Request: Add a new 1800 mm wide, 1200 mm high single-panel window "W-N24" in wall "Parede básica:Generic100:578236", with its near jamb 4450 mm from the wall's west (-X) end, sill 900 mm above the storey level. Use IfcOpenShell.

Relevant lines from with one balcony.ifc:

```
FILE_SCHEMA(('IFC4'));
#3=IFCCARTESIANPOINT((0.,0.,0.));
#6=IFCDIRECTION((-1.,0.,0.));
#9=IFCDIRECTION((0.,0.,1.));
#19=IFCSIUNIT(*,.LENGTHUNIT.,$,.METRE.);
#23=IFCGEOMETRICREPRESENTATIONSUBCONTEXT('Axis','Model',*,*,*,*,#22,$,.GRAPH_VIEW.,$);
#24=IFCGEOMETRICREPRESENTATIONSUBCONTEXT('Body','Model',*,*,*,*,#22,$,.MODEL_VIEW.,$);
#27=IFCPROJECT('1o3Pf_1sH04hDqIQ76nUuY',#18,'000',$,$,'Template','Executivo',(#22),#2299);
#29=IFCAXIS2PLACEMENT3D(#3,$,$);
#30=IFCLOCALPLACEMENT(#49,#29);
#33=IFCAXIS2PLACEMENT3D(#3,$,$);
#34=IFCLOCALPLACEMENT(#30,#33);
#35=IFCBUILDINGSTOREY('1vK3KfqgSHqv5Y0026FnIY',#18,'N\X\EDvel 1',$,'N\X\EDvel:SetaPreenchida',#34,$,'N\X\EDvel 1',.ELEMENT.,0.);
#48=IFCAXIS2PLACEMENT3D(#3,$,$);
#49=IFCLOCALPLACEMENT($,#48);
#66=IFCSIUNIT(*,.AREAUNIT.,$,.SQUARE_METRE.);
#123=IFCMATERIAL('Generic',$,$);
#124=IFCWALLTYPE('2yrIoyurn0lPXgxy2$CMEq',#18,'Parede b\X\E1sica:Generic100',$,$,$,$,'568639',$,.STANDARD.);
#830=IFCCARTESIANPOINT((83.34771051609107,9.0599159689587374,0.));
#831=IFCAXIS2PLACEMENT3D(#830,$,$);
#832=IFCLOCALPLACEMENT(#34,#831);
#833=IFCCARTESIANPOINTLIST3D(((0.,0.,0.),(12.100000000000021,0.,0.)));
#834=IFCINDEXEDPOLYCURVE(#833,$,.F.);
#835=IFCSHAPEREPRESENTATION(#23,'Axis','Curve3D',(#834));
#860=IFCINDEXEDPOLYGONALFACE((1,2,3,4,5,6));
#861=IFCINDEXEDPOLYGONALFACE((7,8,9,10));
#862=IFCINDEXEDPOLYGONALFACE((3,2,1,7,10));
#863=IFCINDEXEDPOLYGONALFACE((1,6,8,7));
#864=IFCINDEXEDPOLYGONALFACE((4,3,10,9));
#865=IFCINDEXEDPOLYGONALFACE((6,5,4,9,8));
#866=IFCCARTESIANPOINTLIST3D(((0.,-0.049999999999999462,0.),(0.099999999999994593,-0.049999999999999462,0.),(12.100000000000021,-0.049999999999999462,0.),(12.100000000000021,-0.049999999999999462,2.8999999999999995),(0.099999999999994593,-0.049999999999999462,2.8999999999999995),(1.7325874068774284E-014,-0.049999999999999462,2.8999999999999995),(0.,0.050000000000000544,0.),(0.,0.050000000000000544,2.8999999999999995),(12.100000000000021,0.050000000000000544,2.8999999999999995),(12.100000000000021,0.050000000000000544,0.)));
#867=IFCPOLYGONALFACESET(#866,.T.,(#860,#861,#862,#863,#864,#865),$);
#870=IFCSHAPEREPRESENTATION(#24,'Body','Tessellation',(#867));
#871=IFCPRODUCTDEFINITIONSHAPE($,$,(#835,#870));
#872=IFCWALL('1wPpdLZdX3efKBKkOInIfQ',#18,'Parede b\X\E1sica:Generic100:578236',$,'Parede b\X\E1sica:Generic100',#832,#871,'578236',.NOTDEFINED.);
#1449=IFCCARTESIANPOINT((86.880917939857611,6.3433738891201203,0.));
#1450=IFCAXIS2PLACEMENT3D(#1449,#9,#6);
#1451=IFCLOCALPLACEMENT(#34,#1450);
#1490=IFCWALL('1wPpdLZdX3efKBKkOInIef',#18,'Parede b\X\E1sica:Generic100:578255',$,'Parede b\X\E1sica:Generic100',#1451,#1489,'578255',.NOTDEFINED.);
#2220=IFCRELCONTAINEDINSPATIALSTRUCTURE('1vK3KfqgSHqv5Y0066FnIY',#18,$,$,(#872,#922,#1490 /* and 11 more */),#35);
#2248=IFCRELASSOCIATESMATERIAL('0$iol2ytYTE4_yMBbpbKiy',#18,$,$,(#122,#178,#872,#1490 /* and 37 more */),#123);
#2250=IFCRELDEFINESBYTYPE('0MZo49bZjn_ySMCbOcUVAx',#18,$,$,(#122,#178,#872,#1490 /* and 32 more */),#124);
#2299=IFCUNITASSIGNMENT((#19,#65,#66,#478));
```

```python
import numpy as np
import ifcopenshell
import ifcopenshell.api.feature
import ifcopenshell.api.geometry
import ifcopenshell.api.root
import ifcopenshell.api.spatial
import ifcopenshell.geom
import ifcopenshell.util.element
import ifcopenshell.util.placement
import ifcopenshell.util.representation
import ifcopenshell.util.shape
import ifcopenshell.util.unit

model = ifcopenshell.open("with one balcony.ifc")
unit_scale = ifcopenshell.util.unit.calculate_unit_scale(model)
settings = ifcopenshell.geom.settings()


def volume(element):
    """Net volume in cubic metres, openings subtracted."""
    shape = ifcopenshell.geom.create_shape(settings, element)
    return ifcopenshell.util.shape.get_volume(shape.geometry)


wall = model.by_guid("1wPpdLZdX3efKBKkOInIfQ")
storey = ifcopenshell.util.element.get_container(wall, ifc_class="IfcBuildingStorey")
context = ifcopenshell.util.representation.get_context(model, "Model", "Body", "MODEL_VIEW")
before = volume(wall)

width, height, from_end, sill = 1.8, 1.2, 4.45, 0.9  # metres

# The wall runs along its own X axis, and the end named is its -X end.
wall_shape = ifcopenshell.geom.create_shape(settings, wall)
x, y, z = ifcopenshell.util.shape.get_vertices(wall_shape.geometry).T
start = x.min() + from_end
face, thickness = float(y.min()), float(y.max() - y.min())
wall_matrix = ifcopenshell.util.placement.get_local_placement(wall.ObjectPlacement)
level = ifcopenshell.util.placement.get_local_placement(storey.ObjectPlacement)[2, 3]


def in_wall(x, y):
    """Placement at x, y metres in the wall's axes, at sill height."""
    matrix = wall_matrix.copy()
    matrix[:, 3] = wall_matrix @ np.array([x / unit_scale, y / unit_scale, 0.0, 1.0])
    matrix[2, 3] = level + sill / unit_scale
    return matrix


# Opening: a box that overshoots both wall faces by 50 mm.
opening = ifcopenshell.api.root.create_entity(model, ifc_class="IfcOpeningElement", predefined_type="OPENING")
box = ifcopenshell.api.geometry.add_wall_representation(
    model, context=context, length=width, height=height, thickness=thickness + 0.1
)
ifcopenshell.api.geometry.assign_representation(model, product=opening, representation=box)
ifcopenshell.api.geometry.edit_object_placement(model, product=opening, matrix=in_wall(start, face - 0.05), is_si=False)
ifcopenshell.api.feature.add_feature(model, feature=opening, element=wall)

window = ifcopenshell.api.root.create_entity(model, ifc_class="IfcWindow", name="W-N24", predefined_type="WINDOW")
window.OverallWidth, window.OverallHeight = width / unit_scale, height / unit_scale
window.PartitioningType = "SINGLE_PANEL"
body = ifcopenshell.api.geometry.add_window_representation(
    model,
    context=context,
    overall_width=window.OverallWidth,
    overall_height=window.OverallHeight,
    partition_type="SINGLE_PANEL",
)
ifcopenshell.api.geometry.assign_representation(model, product=window, representation=body)
ifcopenshell.api.spatial.assign_container(model, products=[window], relating_structure=storey)
ifcopenshell.api.feature.add_filling(model, opening=opening, element=window)

# Centre the window in the wall's thickness.
ifcopenshell.api.geometry.edit_object_placement(model, product=window, matrix=in_wall(start, face), is_si=False)
window_shape = ifcopenshell.geom.create_shape(settings, window)
depth = ifcopenshell.util.shape.get_vertices(window_shape.geometry)[:, 1]
offset = face + thickness / 2 - (depth.min() + depth.max()) / 2
ifcopenshell.api.geometry.edit_object_placement(model, product=window, matrix=in_wall(start, offset), is_si=False)

after = volume(wall)

print(f"wall volume {before:.3f} -> {after:.3f} m3")

model.write("with one balcony_v2.ifc")
```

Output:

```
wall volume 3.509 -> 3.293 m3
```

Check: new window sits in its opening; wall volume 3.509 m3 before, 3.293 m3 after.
